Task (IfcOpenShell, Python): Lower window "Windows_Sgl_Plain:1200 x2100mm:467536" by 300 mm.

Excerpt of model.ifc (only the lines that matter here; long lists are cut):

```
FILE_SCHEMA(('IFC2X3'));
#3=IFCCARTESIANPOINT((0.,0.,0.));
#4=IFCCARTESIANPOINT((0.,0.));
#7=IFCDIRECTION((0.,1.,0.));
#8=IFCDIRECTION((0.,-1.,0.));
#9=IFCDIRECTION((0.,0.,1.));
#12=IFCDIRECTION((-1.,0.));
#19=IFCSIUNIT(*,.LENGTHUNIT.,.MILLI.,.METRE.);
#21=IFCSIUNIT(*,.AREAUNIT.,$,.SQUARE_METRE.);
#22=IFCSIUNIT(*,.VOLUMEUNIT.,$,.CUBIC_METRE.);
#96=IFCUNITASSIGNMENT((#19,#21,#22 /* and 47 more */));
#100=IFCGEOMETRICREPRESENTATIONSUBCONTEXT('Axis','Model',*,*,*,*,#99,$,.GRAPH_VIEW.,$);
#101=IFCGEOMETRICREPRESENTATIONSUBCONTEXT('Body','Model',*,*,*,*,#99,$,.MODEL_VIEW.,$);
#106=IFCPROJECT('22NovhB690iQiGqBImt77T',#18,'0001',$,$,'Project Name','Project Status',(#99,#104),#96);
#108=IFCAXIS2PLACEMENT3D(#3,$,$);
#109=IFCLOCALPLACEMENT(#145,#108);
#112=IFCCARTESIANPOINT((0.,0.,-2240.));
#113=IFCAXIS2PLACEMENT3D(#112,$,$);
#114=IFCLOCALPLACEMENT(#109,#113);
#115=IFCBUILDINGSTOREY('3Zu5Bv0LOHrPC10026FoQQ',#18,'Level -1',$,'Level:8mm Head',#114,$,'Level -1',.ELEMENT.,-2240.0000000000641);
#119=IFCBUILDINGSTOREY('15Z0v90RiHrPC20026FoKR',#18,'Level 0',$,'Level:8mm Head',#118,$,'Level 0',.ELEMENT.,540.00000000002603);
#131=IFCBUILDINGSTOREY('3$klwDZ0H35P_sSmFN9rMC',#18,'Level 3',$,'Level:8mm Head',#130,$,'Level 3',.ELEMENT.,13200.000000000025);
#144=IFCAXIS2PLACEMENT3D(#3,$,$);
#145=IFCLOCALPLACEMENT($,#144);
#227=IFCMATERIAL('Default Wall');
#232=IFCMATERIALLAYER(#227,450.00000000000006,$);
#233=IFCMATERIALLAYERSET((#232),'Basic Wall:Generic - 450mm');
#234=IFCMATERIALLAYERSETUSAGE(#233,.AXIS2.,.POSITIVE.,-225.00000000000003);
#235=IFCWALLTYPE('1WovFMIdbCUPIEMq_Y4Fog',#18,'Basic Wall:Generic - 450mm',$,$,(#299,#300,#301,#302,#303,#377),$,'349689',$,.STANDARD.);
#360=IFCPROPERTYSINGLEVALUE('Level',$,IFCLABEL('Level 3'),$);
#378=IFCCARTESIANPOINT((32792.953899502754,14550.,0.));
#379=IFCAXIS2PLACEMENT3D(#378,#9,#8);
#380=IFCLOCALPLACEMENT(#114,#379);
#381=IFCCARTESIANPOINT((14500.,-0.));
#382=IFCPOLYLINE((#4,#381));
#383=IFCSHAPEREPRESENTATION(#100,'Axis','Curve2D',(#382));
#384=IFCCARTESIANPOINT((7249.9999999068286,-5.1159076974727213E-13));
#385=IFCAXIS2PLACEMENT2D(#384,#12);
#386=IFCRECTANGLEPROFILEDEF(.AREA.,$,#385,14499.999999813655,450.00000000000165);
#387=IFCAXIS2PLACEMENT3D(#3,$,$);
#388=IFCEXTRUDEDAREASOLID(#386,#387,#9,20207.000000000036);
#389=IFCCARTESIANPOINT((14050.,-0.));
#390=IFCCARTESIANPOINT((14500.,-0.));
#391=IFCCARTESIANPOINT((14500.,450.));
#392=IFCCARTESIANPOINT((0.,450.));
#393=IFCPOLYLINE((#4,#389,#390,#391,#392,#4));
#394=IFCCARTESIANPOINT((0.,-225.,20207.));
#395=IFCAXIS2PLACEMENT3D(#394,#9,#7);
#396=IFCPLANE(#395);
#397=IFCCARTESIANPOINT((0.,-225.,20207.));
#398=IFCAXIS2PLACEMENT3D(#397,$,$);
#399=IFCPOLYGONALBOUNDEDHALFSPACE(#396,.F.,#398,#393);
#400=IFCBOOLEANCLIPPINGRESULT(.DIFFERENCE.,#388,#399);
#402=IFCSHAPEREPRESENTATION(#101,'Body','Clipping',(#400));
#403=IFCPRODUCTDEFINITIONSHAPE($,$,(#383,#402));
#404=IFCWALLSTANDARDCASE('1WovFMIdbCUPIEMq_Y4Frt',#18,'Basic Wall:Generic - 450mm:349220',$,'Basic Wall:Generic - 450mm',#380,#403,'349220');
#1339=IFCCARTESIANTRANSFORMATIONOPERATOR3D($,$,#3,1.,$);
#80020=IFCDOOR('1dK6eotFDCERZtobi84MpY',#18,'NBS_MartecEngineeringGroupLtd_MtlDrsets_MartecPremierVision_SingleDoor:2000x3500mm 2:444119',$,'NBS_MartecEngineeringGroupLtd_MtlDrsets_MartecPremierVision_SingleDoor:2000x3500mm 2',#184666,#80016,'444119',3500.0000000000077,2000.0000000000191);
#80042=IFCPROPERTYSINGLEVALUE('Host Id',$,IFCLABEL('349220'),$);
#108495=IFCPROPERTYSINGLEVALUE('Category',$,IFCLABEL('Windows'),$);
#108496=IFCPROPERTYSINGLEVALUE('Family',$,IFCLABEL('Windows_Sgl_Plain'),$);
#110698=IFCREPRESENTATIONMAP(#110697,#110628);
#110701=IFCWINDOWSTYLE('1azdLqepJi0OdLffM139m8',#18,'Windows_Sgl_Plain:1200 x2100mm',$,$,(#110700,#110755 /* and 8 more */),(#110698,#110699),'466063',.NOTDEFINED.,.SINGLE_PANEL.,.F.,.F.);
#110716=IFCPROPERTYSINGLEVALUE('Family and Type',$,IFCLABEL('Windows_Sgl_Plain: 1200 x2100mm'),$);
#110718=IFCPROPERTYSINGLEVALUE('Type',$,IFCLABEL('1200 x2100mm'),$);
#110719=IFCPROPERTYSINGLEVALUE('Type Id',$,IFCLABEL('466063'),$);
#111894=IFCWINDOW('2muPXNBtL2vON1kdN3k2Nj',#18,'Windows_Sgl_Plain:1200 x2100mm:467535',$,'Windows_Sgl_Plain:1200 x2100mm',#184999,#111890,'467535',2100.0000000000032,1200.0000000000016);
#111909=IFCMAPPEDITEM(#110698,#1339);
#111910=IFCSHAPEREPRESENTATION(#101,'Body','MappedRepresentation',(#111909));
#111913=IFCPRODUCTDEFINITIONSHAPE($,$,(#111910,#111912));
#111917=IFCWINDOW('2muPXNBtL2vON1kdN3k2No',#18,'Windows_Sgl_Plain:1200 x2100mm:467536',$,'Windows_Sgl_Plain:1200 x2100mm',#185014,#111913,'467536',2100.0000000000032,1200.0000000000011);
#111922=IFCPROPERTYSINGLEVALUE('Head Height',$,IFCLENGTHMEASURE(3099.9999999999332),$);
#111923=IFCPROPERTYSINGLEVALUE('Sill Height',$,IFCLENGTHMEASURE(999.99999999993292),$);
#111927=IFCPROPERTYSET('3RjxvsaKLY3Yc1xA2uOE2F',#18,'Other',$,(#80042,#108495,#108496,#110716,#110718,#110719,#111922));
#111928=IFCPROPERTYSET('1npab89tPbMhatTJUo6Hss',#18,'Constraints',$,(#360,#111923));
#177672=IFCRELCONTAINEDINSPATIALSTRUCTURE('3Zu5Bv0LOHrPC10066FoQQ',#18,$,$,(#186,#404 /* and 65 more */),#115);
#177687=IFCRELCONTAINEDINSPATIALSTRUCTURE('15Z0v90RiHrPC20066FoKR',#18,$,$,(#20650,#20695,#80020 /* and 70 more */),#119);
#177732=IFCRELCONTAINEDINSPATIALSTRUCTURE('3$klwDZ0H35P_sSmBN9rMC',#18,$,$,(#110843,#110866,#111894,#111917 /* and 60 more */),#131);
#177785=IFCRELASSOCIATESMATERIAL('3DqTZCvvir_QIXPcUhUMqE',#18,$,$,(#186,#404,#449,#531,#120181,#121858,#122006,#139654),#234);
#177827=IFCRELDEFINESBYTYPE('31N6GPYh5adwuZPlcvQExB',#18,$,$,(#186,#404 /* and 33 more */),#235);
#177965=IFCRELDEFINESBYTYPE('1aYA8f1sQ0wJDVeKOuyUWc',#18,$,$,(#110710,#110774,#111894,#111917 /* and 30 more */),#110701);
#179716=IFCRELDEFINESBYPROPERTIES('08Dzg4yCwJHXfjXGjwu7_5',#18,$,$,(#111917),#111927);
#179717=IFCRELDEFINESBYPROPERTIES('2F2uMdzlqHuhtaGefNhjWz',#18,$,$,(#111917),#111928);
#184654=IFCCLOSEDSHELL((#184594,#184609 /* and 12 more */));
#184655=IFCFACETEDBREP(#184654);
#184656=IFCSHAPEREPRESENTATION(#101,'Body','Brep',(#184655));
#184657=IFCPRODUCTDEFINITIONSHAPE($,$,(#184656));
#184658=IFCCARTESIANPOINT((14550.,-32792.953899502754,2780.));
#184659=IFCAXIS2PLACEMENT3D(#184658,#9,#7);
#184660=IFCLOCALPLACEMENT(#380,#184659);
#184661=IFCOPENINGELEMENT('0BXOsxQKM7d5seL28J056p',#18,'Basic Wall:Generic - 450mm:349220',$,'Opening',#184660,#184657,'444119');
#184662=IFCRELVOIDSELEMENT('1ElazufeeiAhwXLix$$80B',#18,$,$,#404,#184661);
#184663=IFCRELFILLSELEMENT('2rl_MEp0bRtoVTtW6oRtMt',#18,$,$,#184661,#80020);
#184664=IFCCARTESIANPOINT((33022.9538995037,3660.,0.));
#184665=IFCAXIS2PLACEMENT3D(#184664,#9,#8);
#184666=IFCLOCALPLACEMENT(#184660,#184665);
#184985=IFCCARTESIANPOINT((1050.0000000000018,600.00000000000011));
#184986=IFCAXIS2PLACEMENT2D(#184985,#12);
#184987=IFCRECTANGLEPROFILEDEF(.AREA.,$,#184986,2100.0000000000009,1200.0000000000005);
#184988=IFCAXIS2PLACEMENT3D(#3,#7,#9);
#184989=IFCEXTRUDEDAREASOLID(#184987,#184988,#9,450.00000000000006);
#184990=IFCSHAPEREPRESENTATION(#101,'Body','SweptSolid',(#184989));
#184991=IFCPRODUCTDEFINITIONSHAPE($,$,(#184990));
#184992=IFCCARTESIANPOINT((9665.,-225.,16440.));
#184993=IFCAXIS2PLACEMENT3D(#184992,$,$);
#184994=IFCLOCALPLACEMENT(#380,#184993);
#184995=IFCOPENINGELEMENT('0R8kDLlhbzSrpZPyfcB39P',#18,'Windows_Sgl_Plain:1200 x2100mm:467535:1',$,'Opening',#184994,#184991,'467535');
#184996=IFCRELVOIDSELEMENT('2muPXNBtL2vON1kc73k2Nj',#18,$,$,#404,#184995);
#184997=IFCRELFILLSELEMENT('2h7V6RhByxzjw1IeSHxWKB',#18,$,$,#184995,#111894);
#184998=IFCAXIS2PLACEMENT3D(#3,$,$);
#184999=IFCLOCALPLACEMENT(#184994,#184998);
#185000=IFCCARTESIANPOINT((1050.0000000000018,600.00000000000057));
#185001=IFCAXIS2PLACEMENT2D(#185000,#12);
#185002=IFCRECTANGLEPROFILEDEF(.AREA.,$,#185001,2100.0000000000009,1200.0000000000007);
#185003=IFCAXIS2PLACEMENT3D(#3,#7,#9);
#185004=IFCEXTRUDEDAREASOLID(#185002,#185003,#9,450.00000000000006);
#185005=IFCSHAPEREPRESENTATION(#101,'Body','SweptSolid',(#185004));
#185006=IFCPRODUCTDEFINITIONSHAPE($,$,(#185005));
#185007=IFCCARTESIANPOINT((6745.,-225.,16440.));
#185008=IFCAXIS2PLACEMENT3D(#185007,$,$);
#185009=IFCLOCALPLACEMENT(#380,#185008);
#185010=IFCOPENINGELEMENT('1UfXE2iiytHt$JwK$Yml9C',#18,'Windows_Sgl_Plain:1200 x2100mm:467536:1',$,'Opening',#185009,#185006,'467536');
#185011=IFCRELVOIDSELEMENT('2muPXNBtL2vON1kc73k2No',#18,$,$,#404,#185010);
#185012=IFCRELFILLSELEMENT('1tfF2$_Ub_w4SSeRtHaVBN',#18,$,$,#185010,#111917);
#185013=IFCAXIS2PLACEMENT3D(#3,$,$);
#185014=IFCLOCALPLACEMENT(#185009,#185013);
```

```python
import numpy as np
import ifcopenshell
import ifcopenshell.api.geometry
import ifcopenshell.api.pset
import ifcopenshell.util.element
import ifcopenshell.util.placement
import ifcopenshell.util.unit

model = ifcopenshell.open("model.ifc")
unit_scale = ifcopenshell.util.unit.calculate_unit_scale(model)

window = model.by_guid("2muPXNBtL2vON1kdN3k2No")
opening = window.FillsVoids[0].RelatingOpeningElement
dz = -0.3 / unit_scale

shift = np.array([0.0, 0.0, dz])
# The window is placed relative to its opening, so it follows when the opening moves.
matrix = ifcopenshell.util.placement.get_local_placement(opening.ObjectPlacement)
matrix[:3, 3] += shift
ifcopenshell.api.geometry.edit_object_placement(
    model, product=opening, matrix=matrix, is_si=False, should_transform_children=True
)

# Keep the stored heights in step.
pset = model.by_id(ifcopenshell.util.element.get_pset(window, "Other", should_inherit=False)["id"])
ifcopenshell.api.pset.edit_pset(model, pset=pset, properties={
    "Head Height": model.create_entity("IfcLengthMeasure", ifcopenshell.util.element.get_pset(window, "Other", "Head Height") + dz),
})
pset = model.by_id(ifcopenshell.util.element.get_pset(window, "Constraints", should_inherit=False)["id"])
ifcopenshell.api.pset.edit_pset(model, pset=pset, properties={
    "Sill Height": model.create_entity("IfcLengthMeasure", ifcopenshell.util.element.get_pset(window, "Constraints", "Sill Height") + dz),
})

print(f"moved by {dz * unit_scale:+.3f} m")

model.write("model-out.ifc")
```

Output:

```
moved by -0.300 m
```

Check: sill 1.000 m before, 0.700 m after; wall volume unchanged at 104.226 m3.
